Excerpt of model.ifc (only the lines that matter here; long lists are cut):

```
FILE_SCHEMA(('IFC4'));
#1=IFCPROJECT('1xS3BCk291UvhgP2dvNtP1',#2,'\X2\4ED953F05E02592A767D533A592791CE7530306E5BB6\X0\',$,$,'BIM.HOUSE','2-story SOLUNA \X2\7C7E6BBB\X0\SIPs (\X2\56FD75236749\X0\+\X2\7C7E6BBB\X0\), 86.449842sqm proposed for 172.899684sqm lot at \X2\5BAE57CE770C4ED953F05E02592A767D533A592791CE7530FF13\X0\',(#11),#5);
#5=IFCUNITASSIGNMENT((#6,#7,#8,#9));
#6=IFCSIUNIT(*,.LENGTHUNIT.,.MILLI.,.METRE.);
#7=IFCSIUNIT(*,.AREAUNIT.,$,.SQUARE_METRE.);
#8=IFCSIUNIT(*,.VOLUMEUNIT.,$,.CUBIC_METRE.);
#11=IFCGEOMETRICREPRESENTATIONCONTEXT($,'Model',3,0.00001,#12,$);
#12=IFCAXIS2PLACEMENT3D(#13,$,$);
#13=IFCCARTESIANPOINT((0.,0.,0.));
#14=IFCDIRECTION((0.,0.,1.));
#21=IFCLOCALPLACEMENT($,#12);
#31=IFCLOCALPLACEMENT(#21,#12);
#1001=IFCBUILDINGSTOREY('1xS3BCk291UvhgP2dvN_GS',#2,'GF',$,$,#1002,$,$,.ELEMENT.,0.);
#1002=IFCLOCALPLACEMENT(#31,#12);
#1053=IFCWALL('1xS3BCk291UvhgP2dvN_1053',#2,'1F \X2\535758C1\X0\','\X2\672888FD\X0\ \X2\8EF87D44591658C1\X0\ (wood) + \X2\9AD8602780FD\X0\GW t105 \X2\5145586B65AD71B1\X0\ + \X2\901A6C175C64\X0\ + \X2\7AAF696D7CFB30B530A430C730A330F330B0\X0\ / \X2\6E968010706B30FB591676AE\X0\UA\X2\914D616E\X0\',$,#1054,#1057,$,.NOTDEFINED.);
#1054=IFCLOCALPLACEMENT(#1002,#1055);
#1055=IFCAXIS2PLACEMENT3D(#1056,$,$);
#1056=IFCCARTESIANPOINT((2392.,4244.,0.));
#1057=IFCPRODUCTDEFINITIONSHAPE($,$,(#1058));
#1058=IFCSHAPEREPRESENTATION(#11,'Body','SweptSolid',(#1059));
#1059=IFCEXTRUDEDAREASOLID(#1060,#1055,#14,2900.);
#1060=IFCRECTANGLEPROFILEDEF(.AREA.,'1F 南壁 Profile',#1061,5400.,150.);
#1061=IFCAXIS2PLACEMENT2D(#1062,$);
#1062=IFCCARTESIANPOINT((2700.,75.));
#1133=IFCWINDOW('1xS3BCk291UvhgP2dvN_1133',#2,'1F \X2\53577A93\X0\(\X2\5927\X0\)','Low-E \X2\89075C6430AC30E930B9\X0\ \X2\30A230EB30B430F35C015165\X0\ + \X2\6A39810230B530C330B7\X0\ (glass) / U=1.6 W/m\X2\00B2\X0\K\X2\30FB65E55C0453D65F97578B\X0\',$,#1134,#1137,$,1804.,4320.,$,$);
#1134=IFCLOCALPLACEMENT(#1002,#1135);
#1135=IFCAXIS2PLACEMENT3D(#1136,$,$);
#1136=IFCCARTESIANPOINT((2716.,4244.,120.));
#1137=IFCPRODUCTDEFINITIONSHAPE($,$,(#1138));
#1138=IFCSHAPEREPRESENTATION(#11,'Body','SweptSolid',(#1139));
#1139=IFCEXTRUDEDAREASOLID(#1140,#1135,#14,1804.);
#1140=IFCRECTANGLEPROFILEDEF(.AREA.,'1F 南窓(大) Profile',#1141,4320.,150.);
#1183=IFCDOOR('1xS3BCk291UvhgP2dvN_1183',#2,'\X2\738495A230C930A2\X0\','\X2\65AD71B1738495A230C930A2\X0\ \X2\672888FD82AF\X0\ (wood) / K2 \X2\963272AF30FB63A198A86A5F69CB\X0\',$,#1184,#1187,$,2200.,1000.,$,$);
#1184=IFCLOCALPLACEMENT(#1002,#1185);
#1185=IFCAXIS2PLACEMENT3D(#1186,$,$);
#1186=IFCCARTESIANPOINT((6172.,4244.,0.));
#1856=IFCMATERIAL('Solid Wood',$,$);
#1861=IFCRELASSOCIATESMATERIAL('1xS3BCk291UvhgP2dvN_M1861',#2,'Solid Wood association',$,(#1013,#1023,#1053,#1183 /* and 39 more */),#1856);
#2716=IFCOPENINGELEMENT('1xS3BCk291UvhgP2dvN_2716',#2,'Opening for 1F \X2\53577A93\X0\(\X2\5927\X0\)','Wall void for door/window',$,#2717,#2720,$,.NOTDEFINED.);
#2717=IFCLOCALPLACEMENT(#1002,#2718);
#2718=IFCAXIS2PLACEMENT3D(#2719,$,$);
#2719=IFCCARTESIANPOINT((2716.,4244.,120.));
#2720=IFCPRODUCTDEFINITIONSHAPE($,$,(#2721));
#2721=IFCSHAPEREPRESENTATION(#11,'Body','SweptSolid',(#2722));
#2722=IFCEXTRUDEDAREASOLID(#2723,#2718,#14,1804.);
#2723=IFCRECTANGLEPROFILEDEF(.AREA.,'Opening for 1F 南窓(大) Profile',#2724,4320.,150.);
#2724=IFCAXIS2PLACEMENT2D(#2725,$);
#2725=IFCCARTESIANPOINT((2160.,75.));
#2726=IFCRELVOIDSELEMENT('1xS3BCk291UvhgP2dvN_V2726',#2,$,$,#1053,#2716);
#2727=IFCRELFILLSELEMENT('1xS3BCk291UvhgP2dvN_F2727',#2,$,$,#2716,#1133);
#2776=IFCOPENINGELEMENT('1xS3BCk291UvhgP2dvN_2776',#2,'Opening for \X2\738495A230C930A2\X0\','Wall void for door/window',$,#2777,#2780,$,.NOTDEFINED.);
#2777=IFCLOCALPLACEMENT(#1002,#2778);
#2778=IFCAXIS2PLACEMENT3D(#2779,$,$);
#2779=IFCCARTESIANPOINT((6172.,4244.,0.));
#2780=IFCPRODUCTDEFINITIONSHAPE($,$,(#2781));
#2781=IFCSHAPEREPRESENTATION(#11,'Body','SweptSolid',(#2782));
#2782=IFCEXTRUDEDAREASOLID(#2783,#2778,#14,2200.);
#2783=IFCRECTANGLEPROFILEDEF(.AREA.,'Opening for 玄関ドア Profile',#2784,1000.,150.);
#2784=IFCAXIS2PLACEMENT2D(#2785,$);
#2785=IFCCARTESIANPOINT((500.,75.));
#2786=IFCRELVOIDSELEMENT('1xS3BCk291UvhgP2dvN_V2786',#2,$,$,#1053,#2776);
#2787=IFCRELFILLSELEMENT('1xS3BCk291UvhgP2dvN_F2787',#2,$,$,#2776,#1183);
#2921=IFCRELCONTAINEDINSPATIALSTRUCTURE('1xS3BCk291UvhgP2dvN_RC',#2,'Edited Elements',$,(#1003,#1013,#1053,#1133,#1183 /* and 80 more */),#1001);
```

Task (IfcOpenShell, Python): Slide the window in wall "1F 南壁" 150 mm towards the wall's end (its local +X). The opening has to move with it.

```python
import ifcopenshell
import ifcopenshell.api.geometry
import ifcopenshell.util.placement
import ifcopenshell.util.unit

model = ifcopenshell.open("model.ifc")
unit_scale = ifcopenshell.util.unit.calculate_unit_scale(model)

window = model.by_id(1133)
opening = window.FillsVoids[0].RelatingOpeningElement
wall = opening.VoidsElements[0].RelatingBuildingElement

wall_matrix = ifcopenshell.util.placement.get_local_placement(wall.ObjectPlacement)
shift = wall_matrix[:3, 0] * 0.15 / unit_scale
before = ifcopenshell.util.placement.get_local_placement(window.ObjectPlacement)[:3, 3].copy()

# The window is not placed relative to its opening, so move both.
for product in (opening, window):
    matrix = ifcopenshell.util.placement.get_local_placement(product.ObjectPlacement)
    matrix[:3, 3] += shift
    ifcopenshell.api.geometry.edit_object_placement(model, product=product, matrix=matrix, is_si=False)

after = ifcopenshell.util.placement.get_local_placement(window.ObjectPlacement)[:3, 3]
print("window moved by", (after - before).round(3) + 0.0)

model.write("model-out.ifc")
```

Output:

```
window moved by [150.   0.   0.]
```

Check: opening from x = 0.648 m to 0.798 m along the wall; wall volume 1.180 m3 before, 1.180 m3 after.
